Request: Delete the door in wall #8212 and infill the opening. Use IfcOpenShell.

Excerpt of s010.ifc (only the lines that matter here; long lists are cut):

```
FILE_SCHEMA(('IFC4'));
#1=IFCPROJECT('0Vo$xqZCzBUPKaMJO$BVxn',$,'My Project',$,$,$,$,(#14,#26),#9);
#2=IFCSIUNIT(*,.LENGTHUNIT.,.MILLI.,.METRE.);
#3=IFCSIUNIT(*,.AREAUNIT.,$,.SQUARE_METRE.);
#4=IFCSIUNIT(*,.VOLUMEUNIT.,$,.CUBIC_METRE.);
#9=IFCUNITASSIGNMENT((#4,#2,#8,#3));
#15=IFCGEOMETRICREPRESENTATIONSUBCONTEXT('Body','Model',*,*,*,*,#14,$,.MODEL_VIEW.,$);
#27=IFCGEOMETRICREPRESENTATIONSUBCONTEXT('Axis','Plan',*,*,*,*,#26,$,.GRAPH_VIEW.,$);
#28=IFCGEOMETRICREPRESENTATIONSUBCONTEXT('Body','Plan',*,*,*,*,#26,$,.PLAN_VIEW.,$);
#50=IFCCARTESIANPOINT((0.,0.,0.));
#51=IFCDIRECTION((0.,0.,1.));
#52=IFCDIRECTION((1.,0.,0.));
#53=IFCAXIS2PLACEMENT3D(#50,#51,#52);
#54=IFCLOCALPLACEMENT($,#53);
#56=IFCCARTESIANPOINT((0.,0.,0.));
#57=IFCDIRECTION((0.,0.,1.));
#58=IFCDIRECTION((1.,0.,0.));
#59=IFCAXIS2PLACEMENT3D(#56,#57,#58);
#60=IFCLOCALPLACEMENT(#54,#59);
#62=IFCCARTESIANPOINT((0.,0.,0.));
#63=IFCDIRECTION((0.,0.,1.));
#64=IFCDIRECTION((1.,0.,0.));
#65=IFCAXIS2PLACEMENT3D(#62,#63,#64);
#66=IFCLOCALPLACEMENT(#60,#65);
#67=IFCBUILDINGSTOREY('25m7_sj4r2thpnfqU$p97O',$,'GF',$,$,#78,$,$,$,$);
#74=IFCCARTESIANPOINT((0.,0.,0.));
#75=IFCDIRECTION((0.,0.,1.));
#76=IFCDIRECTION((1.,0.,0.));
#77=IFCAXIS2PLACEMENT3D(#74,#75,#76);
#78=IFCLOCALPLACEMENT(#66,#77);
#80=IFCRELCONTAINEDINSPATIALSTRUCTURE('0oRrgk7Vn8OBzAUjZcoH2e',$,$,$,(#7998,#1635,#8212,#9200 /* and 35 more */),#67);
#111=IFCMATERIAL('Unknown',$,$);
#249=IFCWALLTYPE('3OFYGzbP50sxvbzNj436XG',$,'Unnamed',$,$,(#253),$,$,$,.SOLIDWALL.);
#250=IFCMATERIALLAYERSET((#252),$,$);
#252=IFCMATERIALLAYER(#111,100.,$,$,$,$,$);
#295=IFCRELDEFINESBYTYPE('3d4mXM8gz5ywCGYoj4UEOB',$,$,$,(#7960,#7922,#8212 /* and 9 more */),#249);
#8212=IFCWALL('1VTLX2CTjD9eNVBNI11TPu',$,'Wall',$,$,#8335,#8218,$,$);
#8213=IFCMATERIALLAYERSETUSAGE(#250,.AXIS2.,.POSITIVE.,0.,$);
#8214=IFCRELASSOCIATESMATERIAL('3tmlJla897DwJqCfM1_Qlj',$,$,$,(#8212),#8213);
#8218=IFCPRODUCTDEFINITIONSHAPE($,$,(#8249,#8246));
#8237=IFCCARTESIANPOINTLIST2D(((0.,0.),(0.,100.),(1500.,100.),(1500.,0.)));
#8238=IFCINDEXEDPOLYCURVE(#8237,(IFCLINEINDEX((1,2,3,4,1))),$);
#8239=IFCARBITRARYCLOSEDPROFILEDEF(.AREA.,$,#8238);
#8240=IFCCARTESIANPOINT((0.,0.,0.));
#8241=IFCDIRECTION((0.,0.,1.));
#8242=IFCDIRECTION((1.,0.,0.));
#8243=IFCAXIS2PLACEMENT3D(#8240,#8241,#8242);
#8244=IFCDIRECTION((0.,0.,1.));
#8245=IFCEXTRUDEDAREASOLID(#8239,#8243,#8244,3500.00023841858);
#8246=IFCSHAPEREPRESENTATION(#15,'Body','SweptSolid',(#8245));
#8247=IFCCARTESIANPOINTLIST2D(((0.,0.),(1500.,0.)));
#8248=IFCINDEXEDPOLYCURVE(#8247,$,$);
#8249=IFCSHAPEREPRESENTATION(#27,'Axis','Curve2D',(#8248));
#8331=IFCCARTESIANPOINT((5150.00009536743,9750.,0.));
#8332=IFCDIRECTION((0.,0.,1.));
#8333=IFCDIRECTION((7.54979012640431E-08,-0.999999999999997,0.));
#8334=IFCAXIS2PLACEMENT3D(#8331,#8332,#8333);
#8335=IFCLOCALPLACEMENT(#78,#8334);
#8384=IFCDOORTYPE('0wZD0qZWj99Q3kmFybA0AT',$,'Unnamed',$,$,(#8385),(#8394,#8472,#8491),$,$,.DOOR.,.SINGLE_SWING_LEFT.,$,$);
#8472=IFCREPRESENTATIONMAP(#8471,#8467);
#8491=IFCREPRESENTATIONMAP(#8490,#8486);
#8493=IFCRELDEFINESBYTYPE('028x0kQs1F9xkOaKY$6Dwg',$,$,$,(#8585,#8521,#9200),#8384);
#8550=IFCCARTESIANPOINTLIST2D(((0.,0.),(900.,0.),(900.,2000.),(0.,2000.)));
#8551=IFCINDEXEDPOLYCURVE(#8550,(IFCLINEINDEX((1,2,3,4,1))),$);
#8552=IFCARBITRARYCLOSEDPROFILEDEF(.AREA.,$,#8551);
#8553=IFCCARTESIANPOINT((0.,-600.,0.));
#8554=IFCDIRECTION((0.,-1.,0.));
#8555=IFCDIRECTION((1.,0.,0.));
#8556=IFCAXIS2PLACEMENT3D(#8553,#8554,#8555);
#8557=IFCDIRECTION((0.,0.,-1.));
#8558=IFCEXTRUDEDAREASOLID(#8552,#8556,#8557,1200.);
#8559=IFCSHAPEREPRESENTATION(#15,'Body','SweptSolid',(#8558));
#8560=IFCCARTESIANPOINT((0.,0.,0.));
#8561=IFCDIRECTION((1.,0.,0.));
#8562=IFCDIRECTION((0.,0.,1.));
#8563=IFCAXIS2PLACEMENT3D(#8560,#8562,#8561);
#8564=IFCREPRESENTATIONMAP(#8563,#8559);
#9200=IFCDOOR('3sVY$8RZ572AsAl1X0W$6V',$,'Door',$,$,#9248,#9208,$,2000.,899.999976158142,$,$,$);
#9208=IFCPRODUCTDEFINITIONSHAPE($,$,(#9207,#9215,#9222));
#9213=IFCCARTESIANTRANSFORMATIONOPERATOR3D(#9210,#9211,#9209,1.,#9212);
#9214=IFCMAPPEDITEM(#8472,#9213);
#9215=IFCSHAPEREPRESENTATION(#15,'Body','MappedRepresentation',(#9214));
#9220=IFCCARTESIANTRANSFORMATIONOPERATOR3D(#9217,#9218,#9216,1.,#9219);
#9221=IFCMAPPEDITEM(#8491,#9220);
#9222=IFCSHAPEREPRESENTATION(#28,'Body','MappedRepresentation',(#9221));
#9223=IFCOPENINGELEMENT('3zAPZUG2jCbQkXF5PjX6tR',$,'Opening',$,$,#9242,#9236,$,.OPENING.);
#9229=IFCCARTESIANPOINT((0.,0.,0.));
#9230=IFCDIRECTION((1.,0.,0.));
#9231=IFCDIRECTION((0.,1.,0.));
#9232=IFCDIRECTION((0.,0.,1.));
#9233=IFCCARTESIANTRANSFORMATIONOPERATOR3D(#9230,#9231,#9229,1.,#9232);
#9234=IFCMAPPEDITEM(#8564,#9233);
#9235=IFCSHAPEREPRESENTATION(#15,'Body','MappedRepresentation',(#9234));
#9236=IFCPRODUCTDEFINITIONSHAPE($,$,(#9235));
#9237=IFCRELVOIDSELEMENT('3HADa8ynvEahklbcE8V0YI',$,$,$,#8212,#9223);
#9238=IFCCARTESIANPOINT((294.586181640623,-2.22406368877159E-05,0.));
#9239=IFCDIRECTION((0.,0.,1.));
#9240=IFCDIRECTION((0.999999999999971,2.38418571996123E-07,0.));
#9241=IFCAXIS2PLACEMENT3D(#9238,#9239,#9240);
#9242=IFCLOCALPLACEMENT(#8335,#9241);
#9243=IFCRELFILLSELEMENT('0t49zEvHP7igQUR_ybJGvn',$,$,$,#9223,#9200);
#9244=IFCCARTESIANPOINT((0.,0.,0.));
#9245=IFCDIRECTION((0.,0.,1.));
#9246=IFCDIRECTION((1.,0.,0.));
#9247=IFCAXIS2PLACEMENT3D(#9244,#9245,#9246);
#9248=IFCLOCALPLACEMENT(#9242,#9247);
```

```python
import ifcopenshell
import ifcopenshell.api.feature
import ifcopenshell.api.root
import ifcopenshell.geom
import ifcopenshell.util.shape

model = ifcopenshell.open("s010.ifc")
settings = ifcopenshell.geom.settings()


def volume(element):
    """Net volume in cubic metres, openings subtracted."""
    shape = ifcopenshell.geom.create_shape(settings, element)
    return ifcopenshell.util.shape.get_volume(shape.geometry)


door = model.by_guid("3sVY$8RZ572AsAl1X0W$6V")
opening = door.FillsVoids[0].RelatingOpeningElement
wall = opening.VoidsElements[0].RelatingBuildingElement
before = volume(wall)

ifcopenshell.api.root.remove_product(model, product=door)
ifcopenshell.api.feature.remove_feature(model, feature=opening)

after = volume(wall)

print(f"wall volume {before:.3f} -> {after:.3f} m3")

model.write("s010_v2.ifc")
```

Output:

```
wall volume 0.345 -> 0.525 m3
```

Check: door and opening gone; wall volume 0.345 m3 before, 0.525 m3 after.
